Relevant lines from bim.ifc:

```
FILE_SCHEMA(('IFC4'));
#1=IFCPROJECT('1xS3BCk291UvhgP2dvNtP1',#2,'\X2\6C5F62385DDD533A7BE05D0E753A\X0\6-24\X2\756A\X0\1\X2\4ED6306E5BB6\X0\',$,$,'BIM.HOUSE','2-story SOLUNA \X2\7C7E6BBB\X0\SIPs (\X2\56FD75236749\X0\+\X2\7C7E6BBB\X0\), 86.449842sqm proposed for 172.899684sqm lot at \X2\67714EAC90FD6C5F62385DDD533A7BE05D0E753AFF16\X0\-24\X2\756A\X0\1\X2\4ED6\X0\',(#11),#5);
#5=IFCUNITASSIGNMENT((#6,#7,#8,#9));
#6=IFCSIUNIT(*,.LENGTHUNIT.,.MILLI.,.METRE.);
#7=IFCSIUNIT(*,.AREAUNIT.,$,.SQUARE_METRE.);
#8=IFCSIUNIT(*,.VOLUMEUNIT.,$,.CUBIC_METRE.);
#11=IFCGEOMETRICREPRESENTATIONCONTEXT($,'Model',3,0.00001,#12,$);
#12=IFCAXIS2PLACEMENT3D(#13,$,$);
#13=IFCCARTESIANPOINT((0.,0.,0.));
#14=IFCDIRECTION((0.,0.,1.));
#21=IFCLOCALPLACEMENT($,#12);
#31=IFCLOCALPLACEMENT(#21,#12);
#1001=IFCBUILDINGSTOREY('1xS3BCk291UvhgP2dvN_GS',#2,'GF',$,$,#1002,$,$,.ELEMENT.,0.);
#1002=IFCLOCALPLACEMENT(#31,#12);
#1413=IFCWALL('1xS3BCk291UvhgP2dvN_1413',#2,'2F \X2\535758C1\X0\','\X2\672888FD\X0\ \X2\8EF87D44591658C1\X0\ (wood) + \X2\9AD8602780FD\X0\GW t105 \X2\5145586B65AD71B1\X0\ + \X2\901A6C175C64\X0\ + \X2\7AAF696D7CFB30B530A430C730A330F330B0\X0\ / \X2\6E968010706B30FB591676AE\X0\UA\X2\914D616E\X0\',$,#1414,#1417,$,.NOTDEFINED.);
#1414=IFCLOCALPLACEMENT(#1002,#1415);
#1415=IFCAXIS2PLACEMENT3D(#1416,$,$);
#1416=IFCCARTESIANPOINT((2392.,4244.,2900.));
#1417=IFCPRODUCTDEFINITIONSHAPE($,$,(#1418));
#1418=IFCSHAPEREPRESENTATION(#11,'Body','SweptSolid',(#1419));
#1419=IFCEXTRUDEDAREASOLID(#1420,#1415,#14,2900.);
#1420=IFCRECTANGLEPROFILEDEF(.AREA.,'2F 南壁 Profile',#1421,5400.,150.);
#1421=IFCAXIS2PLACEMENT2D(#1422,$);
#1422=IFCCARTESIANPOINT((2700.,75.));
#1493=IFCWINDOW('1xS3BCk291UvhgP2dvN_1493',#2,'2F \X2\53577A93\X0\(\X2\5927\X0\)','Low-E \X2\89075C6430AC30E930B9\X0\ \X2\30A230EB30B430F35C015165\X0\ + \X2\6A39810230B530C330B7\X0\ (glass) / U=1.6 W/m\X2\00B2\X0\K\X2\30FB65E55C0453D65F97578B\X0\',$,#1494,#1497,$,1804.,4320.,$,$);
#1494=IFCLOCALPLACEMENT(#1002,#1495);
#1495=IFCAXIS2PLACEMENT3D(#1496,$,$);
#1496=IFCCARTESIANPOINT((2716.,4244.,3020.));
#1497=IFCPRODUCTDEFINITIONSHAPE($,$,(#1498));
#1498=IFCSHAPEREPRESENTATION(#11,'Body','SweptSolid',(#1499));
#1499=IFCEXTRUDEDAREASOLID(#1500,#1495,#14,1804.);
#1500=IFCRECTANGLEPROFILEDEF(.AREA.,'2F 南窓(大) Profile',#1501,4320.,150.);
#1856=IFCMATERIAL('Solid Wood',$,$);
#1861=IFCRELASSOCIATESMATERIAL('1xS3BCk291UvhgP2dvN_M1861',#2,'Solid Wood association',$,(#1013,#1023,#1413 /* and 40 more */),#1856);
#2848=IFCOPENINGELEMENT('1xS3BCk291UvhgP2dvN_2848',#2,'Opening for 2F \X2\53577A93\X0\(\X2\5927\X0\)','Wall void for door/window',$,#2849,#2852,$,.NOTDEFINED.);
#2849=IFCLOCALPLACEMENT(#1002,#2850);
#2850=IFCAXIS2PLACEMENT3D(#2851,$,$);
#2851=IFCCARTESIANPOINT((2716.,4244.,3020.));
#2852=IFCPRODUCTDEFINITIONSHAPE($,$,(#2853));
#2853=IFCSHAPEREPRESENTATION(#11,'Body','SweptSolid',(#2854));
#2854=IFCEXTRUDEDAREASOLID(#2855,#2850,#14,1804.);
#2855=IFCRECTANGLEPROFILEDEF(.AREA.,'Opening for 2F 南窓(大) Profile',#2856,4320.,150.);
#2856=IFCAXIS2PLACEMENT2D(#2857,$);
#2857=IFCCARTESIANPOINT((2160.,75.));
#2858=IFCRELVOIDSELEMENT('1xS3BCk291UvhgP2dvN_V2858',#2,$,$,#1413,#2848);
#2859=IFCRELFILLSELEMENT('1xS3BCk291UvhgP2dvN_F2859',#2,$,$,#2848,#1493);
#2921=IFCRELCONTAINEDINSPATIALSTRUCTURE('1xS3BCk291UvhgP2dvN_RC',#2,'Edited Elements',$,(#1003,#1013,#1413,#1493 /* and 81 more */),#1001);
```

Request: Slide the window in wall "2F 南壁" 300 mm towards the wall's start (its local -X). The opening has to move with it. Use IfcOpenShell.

```python
import ifcopenshell
import ifcopenshell.api.geometry
import ifcopenshell.util.placement

model = ifcopenshell.open("bim.ifc")

window = model.by_guid("1xS3BCk291UvhgP2dvN_1493")
opening = window.FillsVoids[0].RelatingOpeningElement
wall = opening.VoidsElements[0].RelatingBuildingElement

wall_matrix = ifcopenshell.util.placement.get_local_placement(wall.ObjectPlacement)
shift = wall_matrix[:3, 0] * -300.0
before = ifcopenshell.util.placement.get_local_placement(window.ObjectPlacement)[:3, 3].copy()

# The window is not placed relative to its opening, so move both.
for product in (opening, window):
    matrix = ifcopenshell.util.placement.get_local_placement(product.ObjectPlacement)
    matrix[:3, 3] += shift
    ifcopenshell.api.geometry.edit_object_placement(model, product=product, matrix=matrix, is_si=False)

after = ifcopenshell.util.placement.get_local_placement(window.ObjectPlacement)[:3, 3]
print("window moved by", (after - before).round(3) + 0.0)

model.write("bim_v2.ifc")
```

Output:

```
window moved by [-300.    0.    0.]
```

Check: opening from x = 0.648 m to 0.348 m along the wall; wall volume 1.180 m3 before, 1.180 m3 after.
